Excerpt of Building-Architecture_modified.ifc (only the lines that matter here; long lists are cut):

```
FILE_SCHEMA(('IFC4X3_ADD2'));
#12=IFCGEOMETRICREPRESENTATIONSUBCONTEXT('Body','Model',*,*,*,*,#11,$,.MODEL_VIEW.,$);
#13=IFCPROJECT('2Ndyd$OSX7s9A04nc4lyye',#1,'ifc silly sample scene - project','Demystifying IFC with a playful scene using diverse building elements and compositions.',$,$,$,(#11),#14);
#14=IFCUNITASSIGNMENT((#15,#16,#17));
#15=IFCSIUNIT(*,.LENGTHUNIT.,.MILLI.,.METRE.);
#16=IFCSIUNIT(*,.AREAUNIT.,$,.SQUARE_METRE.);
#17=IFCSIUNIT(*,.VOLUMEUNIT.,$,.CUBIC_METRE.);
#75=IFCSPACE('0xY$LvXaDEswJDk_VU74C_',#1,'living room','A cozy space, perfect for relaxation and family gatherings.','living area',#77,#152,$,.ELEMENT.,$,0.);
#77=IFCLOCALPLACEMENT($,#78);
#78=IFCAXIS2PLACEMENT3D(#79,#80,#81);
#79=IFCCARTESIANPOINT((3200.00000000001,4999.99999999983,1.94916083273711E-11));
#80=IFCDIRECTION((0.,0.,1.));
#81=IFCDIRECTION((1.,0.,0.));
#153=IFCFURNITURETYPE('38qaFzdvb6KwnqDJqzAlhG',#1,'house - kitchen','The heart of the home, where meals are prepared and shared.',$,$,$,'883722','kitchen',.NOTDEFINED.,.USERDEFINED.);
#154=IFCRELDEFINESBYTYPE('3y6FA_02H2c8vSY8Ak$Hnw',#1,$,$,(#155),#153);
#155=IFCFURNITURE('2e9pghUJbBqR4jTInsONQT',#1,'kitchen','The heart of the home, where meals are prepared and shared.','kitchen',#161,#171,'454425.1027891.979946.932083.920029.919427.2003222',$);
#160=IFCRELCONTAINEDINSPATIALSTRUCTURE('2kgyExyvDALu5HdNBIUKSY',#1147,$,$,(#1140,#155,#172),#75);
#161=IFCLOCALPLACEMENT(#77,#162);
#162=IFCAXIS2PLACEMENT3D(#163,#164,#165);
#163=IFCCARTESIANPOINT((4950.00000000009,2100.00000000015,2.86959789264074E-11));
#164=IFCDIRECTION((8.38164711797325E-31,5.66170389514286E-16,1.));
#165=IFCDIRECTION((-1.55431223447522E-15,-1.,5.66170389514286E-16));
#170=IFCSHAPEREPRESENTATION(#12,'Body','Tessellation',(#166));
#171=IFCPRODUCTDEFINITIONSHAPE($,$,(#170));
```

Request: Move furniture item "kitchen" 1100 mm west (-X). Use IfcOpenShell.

```python
import ifcopenshell
import ifcopenshell.api.geometry
import ifcopenshell.util.placement
import ifcopenshell.util.unit

model = ifcopenshell.open("Building-Architecture_modified.ifc")
unit_scale = ifcopenshell.util.unit.calculate_unit_scale(model)

item = model.by_guid("2e9pghUJbBqR4jTInsONQT")
matrix = ifcopenshell.util.placement.get_local_placement(item.ObjectPlacement)
matrix[0, 3] -= 1.1 / unit_scale
ifcopenshell.api.geometry.edit_object_placement(model, product=item, matrix=matrix, is_si=False)

print(ifcopenshell.util.placement.get_local_placement(item.ObjectPlacement).round(3) + 0.0)

model.write("Building-Architecture_modified-out.ifc")
```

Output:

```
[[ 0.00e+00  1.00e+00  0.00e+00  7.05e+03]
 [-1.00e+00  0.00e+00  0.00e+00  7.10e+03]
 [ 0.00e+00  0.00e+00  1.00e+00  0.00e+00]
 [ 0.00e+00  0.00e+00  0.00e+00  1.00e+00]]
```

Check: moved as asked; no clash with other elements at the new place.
